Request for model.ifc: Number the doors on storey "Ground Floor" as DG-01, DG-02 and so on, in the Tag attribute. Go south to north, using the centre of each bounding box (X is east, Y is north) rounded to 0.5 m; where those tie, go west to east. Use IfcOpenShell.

First a look at what the model holds.

```python
import ifcopenshell
import ifcopenshell.util.element
import ifcopenshell.util.placement

model = ifcopenshell.open("model.ifc")
print(model.schema)
storey = next(s for s in model.by_type("IfcBuildingStorey") if s.Name == "Ground Floor")
doors = [e for e in ifcopenshell.util.element.get_decomposition(storey) if e.is_a("IfcDoor")]
for e in sorted(doors, key=lambda e: e.id()):
    origin = ifcopenshell.util.placement.get_local_placement(e.ObjectPlacement)[:3, 3]
    print(e.id(), e.Tag, e.Name, origin.round(2) + 0.0, sep=" | ")
```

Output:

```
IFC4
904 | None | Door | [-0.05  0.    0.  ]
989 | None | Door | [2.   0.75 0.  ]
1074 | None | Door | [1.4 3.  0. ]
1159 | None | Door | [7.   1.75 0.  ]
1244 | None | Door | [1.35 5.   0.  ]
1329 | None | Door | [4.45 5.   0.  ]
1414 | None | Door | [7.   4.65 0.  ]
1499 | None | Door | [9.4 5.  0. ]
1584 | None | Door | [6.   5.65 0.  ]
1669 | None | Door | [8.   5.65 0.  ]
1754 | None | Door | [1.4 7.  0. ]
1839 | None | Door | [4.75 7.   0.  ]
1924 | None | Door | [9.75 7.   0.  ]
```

```python
import ifcopenshell
import ifcopenshell.geom
import ifcopenshell.util.element
import ifcopenshell.util.shape

model = ifcopenshell.open("model.ifc")
settings = ifcopenshell.geom.settings()
settings.set("use-world-coords", True)


def centre(element):
    shape = ifcopenshell.geom.create_shape(settings, element)
    return ifcopenshell.util.shape.get_bbox_centroid(shape.geometry)


storey = next(s for s in model.by_type("IfcBuildingStorey") if s.Name == "Ground Floor")
doors = [e for e in ifcopenshell.util.element.get_decomposition(storey) if e.is_a("IfcDoor")]

# Insertion points can sit at a corner or the storey origin, so sort by the geometry (in metres).
centres = {e: centre(e) for e in doors}
doors.sort(key=lambda e: (round(centres[e][1] / 0.5), centres[e][0]))

for i, e in enumerate(doors, start=1):
    number = f"DG-{i:02d}"
    e.Tag = number
    print(e.id(), number)

model.write("model_v2.ifc")
```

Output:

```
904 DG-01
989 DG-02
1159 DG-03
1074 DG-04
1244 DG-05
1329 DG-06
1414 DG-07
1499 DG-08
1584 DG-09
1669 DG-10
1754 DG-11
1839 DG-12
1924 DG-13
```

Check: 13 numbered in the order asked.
